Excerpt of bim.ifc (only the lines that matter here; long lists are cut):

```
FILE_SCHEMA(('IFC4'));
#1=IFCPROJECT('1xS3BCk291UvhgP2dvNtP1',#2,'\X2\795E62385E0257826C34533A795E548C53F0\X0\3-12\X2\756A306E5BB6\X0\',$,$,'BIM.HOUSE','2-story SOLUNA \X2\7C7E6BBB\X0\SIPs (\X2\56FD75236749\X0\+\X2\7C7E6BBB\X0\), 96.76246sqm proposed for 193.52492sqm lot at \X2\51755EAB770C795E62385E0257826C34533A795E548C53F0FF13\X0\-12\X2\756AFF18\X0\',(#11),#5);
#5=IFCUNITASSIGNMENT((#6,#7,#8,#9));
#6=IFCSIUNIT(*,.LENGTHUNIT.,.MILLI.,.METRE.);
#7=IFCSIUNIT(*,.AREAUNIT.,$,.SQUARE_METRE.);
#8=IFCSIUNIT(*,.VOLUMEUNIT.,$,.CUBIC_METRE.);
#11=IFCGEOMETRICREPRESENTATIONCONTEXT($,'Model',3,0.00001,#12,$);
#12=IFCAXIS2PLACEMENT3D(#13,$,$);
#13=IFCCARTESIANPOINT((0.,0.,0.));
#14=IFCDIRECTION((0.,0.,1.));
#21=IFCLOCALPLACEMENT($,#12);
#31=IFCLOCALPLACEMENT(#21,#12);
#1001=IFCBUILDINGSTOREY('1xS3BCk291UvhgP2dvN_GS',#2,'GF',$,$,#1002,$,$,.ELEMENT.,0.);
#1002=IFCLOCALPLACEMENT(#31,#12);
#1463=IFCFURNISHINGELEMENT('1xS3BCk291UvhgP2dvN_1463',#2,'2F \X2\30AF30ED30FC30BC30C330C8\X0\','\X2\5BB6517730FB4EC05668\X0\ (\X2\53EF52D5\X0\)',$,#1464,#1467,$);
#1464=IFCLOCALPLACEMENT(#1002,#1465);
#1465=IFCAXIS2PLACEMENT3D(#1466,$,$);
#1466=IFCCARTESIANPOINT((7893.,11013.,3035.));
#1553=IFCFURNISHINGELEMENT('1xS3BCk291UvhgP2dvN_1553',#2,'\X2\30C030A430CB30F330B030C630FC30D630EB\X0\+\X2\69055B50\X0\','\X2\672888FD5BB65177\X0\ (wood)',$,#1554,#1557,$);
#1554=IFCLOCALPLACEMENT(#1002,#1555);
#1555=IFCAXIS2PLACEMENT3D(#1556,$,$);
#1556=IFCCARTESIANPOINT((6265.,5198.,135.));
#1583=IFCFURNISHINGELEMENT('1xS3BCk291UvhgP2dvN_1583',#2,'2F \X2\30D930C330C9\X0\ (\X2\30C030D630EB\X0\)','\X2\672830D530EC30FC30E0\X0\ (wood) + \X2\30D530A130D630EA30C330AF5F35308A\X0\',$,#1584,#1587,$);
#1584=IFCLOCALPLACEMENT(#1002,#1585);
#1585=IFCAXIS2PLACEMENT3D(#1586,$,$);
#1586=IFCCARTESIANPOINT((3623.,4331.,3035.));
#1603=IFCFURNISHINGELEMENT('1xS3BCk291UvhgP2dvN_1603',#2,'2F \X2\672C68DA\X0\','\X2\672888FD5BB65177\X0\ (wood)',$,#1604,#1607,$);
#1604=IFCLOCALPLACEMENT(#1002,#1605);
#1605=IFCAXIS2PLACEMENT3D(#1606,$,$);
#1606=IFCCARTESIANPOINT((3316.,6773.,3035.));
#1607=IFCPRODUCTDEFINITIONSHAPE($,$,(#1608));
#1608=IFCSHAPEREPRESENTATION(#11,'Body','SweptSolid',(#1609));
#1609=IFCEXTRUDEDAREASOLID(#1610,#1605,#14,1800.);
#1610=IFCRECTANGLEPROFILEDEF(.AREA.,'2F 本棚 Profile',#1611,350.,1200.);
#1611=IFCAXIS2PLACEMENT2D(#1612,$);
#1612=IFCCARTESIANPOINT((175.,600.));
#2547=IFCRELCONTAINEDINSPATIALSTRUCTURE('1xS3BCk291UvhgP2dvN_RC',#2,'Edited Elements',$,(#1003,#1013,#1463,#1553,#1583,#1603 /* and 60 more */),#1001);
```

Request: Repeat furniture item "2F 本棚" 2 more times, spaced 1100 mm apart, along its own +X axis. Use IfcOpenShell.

```python
import ifcopenshell
import ifcopenshell.api.geometry
import ifcopenshell.api.root
import ifcopenshell.util.element
import ifcopenshell.util.placement

model = ifcopenshell.open("bim.ifc")


def reuse_history(source, copy):
    """copy_class also copies each property set's owner history, people and application; keep the originals."""
    for rel in copy.IsDefinedBy:
        if rel.is_a("IfcRelDefinesByProperties") and (history := rel.RelatingPropertyDefinition.OwnerHistory):
            rel.RelatingPropertyDefinition.OwnerHistory = source.OwnerHistory
            ifcopenshell.util.element.remove_deep2(model, history)


source = model.by_guid("1xS3BCk291UvhgP2dvN_1603")
base = ifcopenshell.util.placement.get_local_placement(source.ObjectPlacement)
step = base[:3, 0] * 1100.0

for i in range(1, 3):
    copy = ifcopenshell.api.root.copy_class(model, product=source)
    copy.Representation = ifcopenshell.util.element.copy_deep(
        model, source.Representation, exclude=["IfcGeometricRepresentationContext", "IfcRepresentationMap"]
    )
    reuse_history(source, copy)
    matrix = base.copy()
    matrix[:3, 3] += i * step
    print("added at", matrix[:3, 3].round(3) + 0.0)
    ifcopenshell.api.geometry.edit_object_placement(model, product=copy, matrix=matrix, is_si=False)

model.write("bim_edited.ifc")
```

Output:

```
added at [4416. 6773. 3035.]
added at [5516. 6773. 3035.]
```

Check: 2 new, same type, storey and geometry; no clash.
